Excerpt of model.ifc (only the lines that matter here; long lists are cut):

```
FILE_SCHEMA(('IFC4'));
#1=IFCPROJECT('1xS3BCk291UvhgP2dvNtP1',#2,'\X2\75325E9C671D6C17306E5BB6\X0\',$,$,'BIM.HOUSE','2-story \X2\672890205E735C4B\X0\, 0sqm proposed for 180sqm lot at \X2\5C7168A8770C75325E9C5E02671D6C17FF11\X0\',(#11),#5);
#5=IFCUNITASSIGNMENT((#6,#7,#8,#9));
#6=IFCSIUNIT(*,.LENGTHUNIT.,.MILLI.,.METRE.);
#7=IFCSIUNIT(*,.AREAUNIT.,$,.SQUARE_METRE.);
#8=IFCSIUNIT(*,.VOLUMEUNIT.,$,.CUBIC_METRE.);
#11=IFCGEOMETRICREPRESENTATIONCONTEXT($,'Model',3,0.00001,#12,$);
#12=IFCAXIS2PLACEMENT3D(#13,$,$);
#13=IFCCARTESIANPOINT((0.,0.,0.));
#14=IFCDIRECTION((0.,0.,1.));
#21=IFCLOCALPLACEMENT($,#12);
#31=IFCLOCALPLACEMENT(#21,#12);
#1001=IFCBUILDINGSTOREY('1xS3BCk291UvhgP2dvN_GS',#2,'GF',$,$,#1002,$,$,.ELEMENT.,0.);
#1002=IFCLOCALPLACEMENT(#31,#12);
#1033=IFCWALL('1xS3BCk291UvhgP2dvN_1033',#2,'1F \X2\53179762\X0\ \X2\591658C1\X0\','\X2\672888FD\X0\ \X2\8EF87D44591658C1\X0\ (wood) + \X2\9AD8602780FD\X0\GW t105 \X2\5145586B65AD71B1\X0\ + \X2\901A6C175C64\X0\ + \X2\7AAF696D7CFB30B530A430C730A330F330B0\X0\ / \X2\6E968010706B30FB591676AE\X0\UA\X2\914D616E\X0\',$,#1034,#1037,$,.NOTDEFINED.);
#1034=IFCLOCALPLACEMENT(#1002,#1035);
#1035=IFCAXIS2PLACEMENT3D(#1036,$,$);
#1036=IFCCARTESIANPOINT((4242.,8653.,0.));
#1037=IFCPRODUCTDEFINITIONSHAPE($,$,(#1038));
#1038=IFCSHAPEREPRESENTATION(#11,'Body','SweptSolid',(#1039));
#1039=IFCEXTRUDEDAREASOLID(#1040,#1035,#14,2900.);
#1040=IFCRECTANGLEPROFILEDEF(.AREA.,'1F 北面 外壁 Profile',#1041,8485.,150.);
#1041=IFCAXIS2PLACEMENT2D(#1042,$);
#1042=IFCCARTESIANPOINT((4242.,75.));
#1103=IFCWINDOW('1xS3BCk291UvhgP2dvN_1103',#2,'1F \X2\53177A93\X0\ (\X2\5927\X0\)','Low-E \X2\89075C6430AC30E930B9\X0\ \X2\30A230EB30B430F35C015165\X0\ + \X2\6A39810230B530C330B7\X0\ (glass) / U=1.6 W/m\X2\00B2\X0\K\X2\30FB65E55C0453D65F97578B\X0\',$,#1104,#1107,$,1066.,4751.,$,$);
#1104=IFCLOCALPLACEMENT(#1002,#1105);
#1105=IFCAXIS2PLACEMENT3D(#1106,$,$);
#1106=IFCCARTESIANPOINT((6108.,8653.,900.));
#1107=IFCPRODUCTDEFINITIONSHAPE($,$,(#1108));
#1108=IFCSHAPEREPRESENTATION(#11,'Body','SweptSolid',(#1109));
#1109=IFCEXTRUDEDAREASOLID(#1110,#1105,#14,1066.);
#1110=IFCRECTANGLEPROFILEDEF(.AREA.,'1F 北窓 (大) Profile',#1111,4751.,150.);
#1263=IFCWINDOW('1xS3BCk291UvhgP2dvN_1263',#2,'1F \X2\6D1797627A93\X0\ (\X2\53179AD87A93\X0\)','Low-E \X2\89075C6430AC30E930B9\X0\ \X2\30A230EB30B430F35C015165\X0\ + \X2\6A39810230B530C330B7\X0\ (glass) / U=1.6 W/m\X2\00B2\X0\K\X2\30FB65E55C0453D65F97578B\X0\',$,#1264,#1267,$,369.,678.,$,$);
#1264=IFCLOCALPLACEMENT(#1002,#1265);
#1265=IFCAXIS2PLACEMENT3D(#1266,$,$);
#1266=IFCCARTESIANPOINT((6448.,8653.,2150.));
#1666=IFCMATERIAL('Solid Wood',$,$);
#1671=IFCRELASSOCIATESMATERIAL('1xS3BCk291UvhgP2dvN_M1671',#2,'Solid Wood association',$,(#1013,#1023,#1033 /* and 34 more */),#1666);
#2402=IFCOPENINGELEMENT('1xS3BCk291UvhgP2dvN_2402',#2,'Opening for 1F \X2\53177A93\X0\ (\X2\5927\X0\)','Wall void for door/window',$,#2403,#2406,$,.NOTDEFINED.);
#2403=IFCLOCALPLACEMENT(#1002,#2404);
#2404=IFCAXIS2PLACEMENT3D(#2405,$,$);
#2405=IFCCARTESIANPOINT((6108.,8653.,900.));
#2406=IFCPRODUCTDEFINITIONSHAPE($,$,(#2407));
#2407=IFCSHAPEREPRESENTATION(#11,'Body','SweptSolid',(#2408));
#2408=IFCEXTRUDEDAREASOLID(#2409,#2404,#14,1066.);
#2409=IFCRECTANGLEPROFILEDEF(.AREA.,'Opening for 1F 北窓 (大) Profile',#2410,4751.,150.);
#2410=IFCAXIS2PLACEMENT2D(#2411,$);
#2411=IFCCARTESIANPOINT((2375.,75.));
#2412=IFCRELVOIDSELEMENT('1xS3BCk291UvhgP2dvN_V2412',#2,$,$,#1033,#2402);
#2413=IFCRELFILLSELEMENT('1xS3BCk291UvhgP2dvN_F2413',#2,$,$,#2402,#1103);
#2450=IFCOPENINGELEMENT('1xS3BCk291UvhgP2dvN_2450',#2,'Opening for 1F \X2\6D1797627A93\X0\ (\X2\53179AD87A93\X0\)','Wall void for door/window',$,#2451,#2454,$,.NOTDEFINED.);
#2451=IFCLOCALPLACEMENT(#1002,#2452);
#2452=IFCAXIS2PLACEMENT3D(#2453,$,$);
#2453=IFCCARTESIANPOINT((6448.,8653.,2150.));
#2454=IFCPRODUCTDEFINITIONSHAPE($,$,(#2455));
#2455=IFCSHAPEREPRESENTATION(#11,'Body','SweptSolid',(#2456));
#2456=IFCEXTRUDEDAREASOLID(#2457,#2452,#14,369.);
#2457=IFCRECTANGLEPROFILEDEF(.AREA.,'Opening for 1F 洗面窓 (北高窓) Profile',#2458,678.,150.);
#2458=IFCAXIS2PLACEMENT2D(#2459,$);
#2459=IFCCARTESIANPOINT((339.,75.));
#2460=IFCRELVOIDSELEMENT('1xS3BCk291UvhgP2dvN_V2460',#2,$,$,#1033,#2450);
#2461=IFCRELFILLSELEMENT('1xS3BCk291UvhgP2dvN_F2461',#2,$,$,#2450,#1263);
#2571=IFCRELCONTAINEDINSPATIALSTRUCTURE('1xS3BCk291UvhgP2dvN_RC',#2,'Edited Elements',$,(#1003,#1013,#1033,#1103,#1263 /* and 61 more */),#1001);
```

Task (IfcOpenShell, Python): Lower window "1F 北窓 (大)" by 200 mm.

```python
import numpy as np
import ifcopenshell
import ifcopenshell.api.geometry
import ifcopenshell.util.placement
import ifcopenshell.util.unit

model = ifcopenshell.open("model.ifc")
unit_scale = ifcopenshell.util.unit.calculate_unit_scale(model)

window = model.by_id(1103)
opening = window.FillsVoids[0].RelatingOpeningElement
dz = -0.2 / unit_scale

shift = np.array([0.0, 0.0, dz])
# The window is not placed relative to its opening, so move both.
for product in (opening, window):
    matrix = ifcopenshell.util.placement.get_local_placement(product.ObjectPlacement)
    matrix[:3, 3] += shift
    ifcopenshell.api.geometry.edit_object_placement(model, product=product, matrix=matrix, is_si=False)

print(f"moved by {dz * unit_scale:+.3f} m")

model.write("model_updated.ifc")
```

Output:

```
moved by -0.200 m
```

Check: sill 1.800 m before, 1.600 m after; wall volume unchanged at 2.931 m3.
